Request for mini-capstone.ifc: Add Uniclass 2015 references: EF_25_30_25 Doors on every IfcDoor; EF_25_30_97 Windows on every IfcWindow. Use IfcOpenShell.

First a look at what the model holds.

```python
import ifcopenshell

model = ifcopenshell.open("mini-capstone.ifc")
print(model.schema)
print("classifications:", [c.Name for c in model.by_type("IfcClassification")])
for ifc_class in ("IfcDoor", "IfcRoof", "IfcStair", "IfcWall", "IfcWindow"):
    print(ifc_class, len(model.by_type(ifc_class)))
```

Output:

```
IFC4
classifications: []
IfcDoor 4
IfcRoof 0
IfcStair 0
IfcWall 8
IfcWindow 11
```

```python
import ifcopenshell
import ifcopenshell.api.classification

model = ifcopenshell.open("mini-capstone.ifc")

system = ifcopenshell.api.classification.add_classification(model, classification="Uniclass 2015")

codes = {
    "IfcDoor": ("EF_25_30_25", "Doors"),
    "IfcWindow": ("EF_25_30_97", "Windows"),
}
for ifc_class, (code, name) in codes.items():
    products = model.by_type(ifc_class)
    ifcopenshell.api.classification.add_reference(
        model, products=products, classification=system, identification=code, name=name
    )
    print(code, len(products))

model.write("mini-capstone_rev.ifc")
```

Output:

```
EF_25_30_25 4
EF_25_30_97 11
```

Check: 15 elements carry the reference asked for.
